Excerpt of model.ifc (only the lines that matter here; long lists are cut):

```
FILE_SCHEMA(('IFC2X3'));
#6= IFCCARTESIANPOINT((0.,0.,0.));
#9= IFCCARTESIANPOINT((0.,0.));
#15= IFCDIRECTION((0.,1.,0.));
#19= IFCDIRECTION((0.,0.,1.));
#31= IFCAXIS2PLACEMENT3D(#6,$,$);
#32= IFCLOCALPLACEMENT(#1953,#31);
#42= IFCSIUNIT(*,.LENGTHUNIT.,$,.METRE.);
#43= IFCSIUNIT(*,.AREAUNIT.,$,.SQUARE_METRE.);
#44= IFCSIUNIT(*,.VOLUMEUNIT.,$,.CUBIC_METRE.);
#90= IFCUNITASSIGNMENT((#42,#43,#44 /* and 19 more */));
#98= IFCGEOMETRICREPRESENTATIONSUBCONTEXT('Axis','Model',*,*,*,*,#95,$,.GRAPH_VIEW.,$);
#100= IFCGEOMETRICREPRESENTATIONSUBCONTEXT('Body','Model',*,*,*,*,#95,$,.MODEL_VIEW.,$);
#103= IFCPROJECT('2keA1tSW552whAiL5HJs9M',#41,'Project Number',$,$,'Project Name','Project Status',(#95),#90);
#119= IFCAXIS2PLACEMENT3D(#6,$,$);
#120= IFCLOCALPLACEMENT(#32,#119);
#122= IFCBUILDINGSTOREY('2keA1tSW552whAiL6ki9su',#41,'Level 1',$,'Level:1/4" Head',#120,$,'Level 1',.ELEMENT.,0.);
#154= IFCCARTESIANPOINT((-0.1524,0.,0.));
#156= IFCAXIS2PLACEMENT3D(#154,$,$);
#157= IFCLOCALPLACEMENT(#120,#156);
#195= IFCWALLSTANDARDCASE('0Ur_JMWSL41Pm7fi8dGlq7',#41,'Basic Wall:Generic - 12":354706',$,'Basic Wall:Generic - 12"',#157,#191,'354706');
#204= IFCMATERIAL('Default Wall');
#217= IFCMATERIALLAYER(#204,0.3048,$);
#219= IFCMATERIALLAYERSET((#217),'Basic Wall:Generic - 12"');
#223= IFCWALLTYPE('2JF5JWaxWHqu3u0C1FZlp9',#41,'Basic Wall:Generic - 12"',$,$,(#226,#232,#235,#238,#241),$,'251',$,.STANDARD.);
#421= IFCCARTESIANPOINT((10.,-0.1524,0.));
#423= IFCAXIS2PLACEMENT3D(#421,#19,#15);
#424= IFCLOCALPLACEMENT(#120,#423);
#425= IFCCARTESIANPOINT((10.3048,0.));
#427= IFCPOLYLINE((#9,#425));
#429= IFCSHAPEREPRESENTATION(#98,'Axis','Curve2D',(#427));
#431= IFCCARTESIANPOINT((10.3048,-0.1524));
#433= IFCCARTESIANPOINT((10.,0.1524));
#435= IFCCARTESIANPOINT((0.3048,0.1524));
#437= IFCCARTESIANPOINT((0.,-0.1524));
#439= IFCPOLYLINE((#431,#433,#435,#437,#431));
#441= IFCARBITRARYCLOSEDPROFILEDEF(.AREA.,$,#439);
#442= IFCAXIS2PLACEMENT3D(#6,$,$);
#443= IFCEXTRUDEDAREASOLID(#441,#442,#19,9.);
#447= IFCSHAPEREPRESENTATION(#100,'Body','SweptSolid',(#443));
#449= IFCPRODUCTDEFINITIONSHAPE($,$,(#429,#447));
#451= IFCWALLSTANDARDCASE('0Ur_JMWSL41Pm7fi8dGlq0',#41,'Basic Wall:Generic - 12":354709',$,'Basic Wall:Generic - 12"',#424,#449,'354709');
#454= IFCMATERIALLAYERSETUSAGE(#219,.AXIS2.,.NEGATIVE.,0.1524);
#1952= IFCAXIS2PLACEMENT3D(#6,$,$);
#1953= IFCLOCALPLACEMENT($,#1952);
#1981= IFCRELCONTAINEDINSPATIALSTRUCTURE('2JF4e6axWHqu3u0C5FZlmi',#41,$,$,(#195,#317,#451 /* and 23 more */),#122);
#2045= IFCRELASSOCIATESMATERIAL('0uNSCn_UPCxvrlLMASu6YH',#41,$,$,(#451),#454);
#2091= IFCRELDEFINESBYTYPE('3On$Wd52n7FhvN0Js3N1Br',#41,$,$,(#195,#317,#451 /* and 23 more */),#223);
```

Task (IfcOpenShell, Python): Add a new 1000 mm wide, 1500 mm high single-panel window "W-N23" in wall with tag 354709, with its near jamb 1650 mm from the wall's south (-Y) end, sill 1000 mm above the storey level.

```python
import numpy as np
import ifcopenshell
import ifcopenshell.api.feature
import ifcopenshell.api.geometry
import ifcopenshell.api.root
import ifcopenshell.api.spatial
import ifcopenshell.api.type
import ifcopenshell.geom
import ifcopenshell.util.element
import ifcopenshell.util.placement
import ifcopenshell.util.representation
import ifcopenshell.util.shape
import ifcopenshell.util.unit

model = ifcopenshell.open("model.ifc")
unit_scale = ifcopenshell.util.unit.calculate_unit_scale(model)
settings = ifcopenshell.geom.settings()


def volume(element):
    """Net volume in cubic metres, openings subtracted."""
    shape = ifcopenshell.geom.create_shape(settings, element)
    return ifcopenshell.util.shape.get_volume(shape.geometry)


wall = model.by_guid("0Ur_JMWSL41Pm7fi8dGlq0")
storey = ifcopenshell.util.element.get_container(wall, ifc_class="IfcBuildingStorey")
context = ifcopenshell.util.representation.get_context(model, "Model", "Body", "MODEL_VIEW")
before = volume(wall)

width, height, from_end, sill = 1, 1.5, 1.65, 1  # metres

# The wall runs along its own X axis, and the end named is its -X end.
wall_shape = ifcopenshell.geom.create_shape(settings, wall)
x, y, z = ifcopenshell.util.shape.get_vertices(wall_shape.geometry).T
start = x.min() + from_end
face, thickness = float(y.min()), float(y.max() - y.min())
wall_matrix = ifcopenshell.util.placement.get_local_placement(wall.ObjectPlacement)
level = ifcopenshell.util.placement.get_local_placement(storey.ObjectPlacement)[2, 3]


def in_wall(x, y):
    """Placement at x, y metres in the wall's axes, at sill height."""
    matrix = wall_matrix.copy()
    matrix[:, 3] = wall_matrix @ np.array([x / unit_scale, y / unit_scale, 0.0, 1.0])
    matrix[2, 3] = level + sill / unit_scale
    return matrix


# Opening: a box that overshoots both wall faces by 50 mm.
opening = ifcopenshell.api.root.create_entity(model, ifc_class="IfcOpeningElement")
box = ifcopenshell.api.geometry.add_wall_representation(
    model, context=context, length=width, height=height, thickness=thickness + 0.1
)
ifcopenshell.api.geometry.assign_representation(model, product=opening, representation=box)
ifcopenshell.api.geometry.edit_object_placement(model, product=opening, matrix=in_wall(start, face - 0.05), is_si=False)
ifcopenshell.api.feature.add_feature(model, feature=opening, element=wall)

window = ifcopenshell.api.root.create_entity(model, ifc_class="IfcWindow", name="W-N23")
window.OverallWidth, window.OverallHeight = width / unit_scale, height / unit_scale
body = ifcopenshell.api.geometry.add_window_representation(
    model,
    context=context,
    overall_width=window.OverallWidth,
    overall_height=window.OverallHeight,
    partition_type="SINGLE_PANEL",
)
ifcopenshell.api.geometry.assign_representation(model, product=window, representation=body)
ifcopenshell.api.spatial.assign_container(model, products=[window], relating_structure=storey)
fills = ifcopenshell.api.feature.add_filling(model, opening=opening, element=window)
fills.OwnerHistory = window.OwnerHistory  # required in IFC2X3

# IFC2X3 keeps the operation on the window style.
style = ifcopenshell.api.root.create_entity(model, ifc_class="IfcWindowStyle", name="W-N23")
style.OperationType, style.ConstructionType = "SINGLE_PANEL", "NOTDEFINED"
style.ParameterTakesPrecedence = style.Sizeable = False
ifcopenshell.api.type.assign_type(model, related_objects=[window], relating_type=style)

# Centre the window in the wall's thickness.
ifcopenshell.api.geometry.edit_object_placement(model, product=window, matrix=in_wall(start, face), is_si=False)
window_shape = ifcopenshell.geom.create_shape(settings, window)
depth = ifcopenshell.util.shape.get_vertices(window_shape.geometry)[:, 1]
offset = face + thickness / 2 - (depth.min() + depth.max()) / 2
ifcopenshell.api.geometry.edit_object_placement(model, product=window, matrix=in_wall(start, offset), is_si=False)

after = volume(wall)

print(f"wall volume {before:.3f} -> {after:.3f} m3")

model.write("model_updated.ifc")
```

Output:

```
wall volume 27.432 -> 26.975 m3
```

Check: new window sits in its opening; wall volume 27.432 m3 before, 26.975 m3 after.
